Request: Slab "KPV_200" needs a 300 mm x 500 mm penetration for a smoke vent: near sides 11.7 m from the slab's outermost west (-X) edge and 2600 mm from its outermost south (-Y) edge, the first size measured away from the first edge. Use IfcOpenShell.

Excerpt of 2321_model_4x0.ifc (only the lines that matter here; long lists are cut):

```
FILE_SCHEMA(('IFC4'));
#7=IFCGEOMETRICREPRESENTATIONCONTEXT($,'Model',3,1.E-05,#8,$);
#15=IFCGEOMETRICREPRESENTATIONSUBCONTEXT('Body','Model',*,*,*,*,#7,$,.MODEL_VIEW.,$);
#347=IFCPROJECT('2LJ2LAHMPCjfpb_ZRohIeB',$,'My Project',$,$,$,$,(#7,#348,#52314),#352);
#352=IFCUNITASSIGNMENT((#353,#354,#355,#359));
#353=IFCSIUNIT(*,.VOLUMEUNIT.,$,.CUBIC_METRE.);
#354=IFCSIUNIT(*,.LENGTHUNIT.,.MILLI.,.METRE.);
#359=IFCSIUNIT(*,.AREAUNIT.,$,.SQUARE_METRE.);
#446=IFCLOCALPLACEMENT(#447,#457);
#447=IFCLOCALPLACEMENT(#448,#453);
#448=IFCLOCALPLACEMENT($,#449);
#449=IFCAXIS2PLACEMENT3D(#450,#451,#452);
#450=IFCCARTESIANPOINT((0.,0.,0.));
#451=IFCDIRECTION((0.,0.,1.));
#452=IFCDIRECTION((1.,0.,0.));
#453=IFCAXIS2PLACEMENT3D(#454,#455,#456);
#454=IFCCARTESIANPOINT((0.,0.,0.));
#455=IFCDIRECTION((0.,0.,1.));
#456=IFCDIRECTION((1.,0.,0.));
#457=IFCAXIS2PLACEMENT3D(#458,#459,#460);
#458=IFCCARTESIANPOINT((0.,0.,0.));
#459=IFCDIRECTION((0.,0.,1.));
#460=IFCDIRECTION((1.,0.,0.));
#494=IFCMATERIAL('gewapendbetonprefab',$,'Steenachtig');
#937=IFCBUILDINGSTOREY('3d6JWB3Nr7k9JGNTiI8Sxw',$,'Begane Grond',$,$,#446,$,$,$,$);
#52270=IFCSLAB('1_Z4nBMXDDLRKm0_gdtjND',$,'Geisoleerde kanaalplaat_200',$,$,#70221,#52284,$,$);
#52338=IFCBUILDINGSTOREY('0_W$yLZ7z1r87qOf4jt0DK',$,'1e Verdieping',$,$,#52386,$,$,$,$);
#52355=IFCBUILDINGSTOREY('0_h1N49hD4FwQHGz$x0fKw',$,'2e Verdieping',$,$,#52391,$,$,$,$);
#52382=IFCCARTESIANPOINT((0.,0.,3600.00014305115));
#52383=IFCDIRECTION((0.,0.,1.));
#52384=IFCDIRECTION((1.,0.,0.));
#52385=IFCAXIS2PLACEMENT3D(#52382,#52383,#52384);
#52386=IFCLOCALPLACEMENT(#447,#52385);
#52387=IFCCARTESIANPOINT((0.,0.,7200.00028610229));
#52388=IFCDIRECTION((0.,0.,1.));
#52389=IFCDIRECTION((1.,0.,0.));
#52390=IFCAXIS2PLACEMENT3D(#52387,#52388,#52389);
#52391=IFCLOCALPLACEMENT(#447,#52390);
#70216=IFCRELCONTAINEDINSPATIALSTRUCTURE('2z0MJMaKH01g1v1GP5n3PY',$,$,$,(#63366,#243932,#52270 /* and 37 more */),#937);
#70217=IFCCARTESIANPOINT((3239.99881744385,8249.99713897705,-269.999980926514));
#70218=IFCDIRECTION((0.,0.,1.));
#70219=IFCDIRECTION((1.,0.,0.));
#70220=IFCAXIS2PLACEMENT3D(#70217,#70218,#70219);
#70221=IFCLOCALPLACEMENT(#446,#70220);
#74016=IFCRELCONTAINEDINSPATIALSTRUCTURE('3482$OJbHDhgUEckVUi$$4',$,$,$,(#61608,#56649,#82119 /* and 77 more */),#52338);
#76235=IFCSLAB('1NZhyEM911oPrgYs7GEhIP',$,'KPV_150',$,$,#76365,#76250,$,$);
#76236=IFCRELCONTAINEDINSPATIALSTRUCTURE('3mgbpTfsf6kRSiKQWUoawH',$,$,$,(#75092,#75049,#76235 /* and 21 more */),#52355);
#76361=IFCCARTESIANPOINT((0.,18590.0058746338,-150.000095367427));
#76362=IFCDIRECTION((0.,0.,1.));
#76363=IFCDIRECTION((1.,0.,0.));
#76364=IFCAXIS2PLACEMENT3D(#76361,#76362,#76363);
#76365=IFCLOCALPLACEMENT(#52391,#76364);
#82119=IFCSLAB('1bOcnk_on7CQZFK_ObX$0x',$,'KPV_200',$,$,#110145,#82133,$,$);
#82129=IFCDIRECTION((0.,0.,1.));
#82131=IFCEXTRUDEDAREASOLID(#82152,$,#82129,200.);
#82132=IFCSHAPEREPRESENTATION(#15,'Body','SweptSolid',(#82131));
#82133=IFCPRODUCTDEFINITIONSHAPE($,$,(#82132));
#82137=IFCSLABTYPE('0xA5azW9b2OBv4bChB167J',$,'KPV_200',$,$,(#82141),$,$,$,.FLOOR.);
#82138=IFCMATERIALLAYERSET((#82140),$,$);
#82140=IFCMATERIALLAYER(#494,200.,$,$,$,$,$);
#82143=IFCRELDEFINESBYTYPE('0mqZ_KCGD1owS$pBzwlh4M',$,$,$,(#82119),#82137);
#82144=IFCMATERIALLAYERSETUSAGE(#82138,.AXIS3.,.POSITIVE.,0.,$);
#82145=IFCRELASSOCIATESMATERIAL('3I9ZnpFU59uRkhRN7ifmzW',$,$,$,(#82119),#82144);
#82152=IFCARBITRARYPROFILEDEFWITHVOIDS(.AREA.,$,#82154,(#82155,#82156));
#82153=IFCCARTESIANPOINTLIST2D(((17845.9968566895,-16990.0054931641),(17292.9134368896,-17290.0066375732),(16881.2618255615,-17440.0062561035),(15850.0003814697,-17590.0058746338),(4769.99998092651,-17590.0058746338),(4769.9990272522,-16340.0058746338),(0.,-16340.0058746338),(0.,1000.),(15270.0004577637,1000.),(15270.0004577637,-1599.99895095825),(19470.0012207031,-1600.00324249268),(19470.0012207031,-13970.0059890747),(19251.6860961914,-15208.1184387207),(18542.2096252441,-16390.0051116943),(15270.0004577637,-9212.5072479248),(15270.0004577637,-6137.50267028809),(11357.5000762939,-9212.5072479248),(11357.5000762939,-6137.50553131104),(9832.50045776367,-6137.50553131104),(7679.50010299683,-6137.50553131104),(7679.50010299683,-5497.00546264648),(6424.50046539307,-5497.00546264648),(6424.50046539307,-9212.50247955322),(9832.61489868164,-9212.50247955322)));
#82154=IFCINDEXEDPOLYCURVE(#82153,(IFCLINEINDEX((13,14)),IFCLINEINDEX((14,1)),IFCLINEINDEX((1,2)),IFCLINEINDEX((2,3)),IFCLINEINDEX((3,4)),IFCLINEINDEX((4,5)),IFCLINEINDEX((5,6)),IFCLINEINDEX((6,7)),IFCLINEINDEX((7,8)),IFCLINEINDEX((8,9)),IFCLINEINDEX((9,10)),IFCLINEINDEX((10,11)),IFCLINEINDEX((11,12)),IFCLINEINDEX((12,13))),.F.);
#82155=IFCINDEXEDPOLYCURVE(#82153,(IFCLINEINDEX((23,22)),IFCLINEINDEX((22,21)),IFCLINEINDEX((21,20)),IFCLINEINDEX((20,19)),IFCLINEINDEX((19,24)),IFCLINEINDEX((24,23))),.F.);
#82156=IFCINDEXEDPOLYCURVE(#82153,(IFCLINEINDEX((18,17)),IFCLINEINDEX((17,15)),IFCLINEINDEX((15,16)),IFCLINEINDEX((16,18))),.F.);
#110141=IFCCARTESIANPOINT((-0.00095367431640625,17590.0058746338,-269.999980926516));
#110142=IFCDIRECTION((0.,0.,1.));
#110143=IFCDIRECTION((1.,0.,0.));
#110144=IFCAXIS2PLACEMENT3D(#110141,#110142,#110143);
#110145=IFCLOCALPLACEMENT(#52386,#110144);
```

```python
import numpy as np
import ifcopenshell
import ifcopenshell.api.feature
import ifcopenshell.api.geometry
import ifcopenshell.api.root
import ifcopenshell.geom
import ifcopenshell.util.placement
import ifcopenshell.util.representation
import ifcopenshell.util.shape
import ifcopenshell.util.unit

model = ifcopenshell.open("2321_model_4x0.ifc")
unit_scale = ifcopenshell.util.unit.calculate_unit_scale(model)
settings = ifcopenshell.geom.settings()


def volume(element):
    """Net volume in cubic metres, openings subtracted."""
    shape = ifcopenshell.geom.create_shape(settings, element)
    return ifcopenshell.util.shape.get_volume(shape.geometry)


slab = model.by_guid("1bOcnk_on7CQZFK_ObX$0x")
before = volume(slab)

# Extent in the slab's own axes, in metres. The edges named are its -X and -Y sides.
slab_shape = ifcopenshell.geom.create_shape(settings, slab)
vertices = ifcopenshell.util.shape.get_vertices(slab_shape.geometry)
x_min, y_min, bottom = vertices.min(axis=0)
top = vertices[:, 2].max()

opening = ifcopenshell.api.root.create_entity(model, ifc_class="IfcOpeningElement", name="Smoke vent opening", predefined_type="OPENING")
context = ifcopenshell.util.representation.get_context(model, "Model", "Body", "MODEL_VIEW")
width, depth = 0.3, 0.5
outline = [(0.0, 0.0), (width, 0.0), (width, depth), (0.0, depth), (0.0, 0.0)]
# Overshoot both faces by 50 mm so the cut is clean.
shape = ifcopenshell.api.geometry.add_slab_representation(
    model, context=context, depth=top - bottom + 0.1, polyline=outline
)
ifcopenshell.api.geometry.assign_representation(model, product=opening, representation=shape)

matrix = ifcopenshell.util.placement.get_local_placement(slab.ObjectPlacement)
matrix[:, 3] = matrix @ np.append(np.array([x_min + 11.7, y_min + 2.6, bottom - 0.05]) / unit_scale, 1.0)
ifcopenshell.api.geometry.edit_object_placement(model, product=opening, matrix=matrix, is_si=False)
ifcopenshell.api.feature.add_feature(model, feature=opening, element=slab)

after = volume(slab)

print(f"slab volume {before:.3f} -> {after:.3f} m3")

model.write("2321_model_4x0_edited.ifc")
```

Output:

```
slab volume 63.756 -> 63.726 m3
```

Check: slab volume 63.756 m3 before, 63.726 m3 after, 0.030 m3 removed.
